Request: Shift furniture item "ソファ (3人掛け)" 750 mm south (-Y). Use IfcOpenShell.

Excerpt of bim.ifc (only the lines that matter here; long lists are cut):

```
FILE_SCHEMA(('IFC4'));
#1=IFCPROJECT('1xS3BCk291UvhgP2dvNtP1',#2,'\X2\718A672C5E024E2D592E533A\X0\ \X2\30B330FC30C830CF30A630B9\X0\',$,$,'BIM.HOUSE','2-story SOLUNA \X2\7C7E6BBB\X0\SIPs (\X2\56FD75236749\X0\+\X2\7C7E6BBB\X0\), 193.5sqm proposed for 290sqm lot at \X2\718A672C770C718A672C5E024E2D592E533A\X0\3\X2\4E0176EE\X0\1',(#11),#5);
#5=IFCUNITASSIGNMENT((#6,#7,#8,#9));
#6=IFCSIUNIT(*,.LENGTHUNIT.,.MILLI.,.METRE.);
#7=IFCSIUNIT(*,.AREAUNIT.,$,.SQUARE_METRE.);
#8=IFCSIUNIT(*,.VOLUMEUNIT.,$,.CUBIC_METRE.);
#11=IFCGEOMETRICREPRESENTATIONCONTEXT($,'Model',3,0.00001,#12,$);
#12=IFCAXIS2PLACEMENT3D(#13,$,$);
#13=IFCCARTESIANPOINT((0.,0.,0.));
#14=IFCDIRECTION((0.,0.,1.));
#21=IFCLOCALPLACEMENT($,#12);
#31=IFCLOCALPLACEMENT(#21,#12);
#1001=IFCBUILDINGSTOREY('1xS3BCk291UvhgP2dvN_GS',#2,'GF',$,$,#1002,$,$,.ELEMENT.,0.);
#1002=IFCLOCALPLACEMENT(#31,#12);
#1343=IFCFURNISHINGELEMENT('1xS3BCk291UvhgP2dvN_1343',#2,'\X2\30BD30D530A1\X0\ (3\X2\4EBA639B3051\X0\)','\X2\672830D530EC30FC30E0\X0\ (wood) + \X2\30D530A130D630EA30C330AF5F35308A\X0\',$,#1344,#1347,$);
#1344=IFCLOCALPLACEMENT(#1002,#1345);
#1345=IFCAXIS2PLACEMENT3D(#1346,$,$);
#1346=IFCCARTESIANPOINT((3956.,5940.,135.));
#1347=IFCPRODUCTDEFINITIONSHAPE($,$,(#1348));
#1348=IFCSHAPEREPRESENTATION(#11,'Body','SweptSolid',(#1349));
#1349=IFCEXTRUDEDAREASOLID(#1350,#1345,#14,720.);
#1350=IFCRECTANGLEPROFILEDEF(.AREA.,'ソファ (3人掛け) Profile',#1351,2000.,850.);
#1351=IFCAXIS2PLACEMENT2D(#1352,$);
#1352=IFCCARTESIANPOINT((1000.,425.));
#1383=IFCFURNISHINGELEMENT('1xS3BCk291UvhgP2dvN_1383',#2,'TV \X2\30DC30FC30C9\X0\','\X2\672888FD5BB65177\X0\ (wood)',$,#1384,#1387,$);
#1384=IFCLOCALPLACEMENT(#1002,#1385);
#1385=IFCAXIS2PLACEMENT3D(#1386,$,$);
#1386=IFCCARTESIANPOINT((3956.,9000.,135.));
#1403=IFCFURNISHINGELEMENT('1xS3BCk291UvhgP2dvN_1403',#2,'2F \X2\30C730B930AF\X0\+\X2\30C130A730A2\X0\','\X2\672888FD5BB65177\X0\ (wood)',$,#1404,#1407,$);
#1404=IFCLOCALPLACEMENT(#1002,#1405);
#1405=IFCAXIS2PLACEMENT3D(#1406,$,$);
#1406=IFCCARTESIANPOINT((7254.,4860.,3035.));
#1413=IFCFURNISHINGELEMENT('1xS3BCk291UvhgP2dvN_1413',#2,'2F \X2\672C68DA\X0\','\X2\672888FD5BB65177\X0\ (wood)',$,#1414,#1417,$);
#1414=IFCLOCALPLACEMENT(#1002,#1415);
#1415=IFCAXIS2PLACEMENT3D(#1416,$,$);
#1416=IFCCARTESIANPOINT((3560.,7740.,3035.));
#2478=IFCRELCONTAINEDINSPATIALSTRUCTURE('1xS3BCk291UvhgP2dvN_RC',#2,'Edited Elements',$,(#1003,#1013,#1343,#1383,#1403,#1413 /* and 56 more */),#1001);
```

```python
import ifcopenshell
import ifcopenshell.api.geometry
import ifcopenshell.util.placement
import ifcopenshell.util.unit

model = ifcopenshell.open("bim.ifc")
unit_scale = ifcopenshell.util.unit.calculate_unit_scale(model)

item = model.by_guid("1xS3BCk291UvhgP2dvN_1343")
matrix = ifcopenshell.util.placement.get_local_placement(item.ObjectPlacement)
matrix[1, 3] -= 0.75 / unit_scale
ifcopenshell.api.geometry.edit_object_placement(model, product=item, matrix=matrix, is_si=False)

print(ifcopenshell.util.placement.get_local_placement(item.ObjectPlacement).round(3) + 0.0)

model.write("bim_updated.ifc")
```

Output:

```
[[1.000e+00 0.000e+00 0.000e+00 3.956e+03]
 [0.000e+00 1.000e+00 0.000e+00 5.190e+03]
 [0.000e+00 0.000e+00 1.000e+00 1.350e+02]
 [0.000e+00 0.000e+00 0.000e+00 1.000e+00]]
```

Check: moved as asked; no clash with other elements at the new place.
